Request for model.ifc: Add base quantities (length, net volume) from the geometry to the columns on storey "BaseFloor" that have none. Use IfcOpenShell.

First a look at what the model holds.

```python
import ifcopenshell
import ifcopenshell.util.element
import ifcopenshell.util.unit

model = ifcopenshell.open("model.ifc")
print(model.schema)
for unit_type in ("LENGTHUNIT", "AREAUNIT", "VOLUMEUNIT"):
    print(unit_type, ifcopenshell.util.unit.calculate_unit_scale(model, unit_type))
storey = next(s for s in model.by_type("IfcBuildingStorey") if s.Name == "BaseFloor")
columns = [e for e in ifcopenshell.util.element.get_decomposition(storey) if e.is_a("IfcColumn")]
for e in sorted(columns, key=lambda e: e.id()):
    print(e.id(), e.is_a(), e.Name, list(ifcopenshell.util.element.get_psets(e, qtos_only=True)), sep=" | ")
```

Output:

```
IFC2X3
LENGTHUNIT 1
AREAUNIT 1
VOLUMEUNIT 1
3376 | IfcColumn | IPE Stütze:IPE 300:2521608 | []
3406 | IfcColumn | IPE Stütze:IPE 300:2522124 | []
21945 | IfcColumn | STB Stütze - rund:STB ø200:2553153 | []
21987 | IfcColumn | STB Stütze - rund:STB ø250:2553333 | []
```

```python
import ifcopenshell
import ifcopenshell.api.pset
import ifcopenshell.geom
import ifcopenshell.util.element
import ifcopenshell.util.shape
import ifcopenshell.util.unit

model = ifcopenshell.open("model.ifc")
unit_scale = ifcopenshell.util.unit.calculate_unit_scale(model)
volume_scale = ifcopenshell.util.unit.calculate_unit_scale(model, "VOLUMEUNIT")
settings = ifcopenshell.geom.settings()

storey = next(s for s in model.by_type("IfcBuildingStorey") if s.Name == "BaseFloor")
columns = [e for e in ifcopenshell.util.element.get_decomposition(storey) if e.is_a("IfcColumn")]

for e in sorted(columns, key=lambda e: e.id()):
    if ifcopenshell.util.element.get_psets(e, qtos_only=True, should_inherit=False):
        continue
    # Geometry comes back in metres, in the element's own axes.
    shape = ifcopenshell.geom.create_shape(settings, e)
    values = {
        "Length": ifcopenshell.util.shape.get_z(shape.geometry) / unit_scale,
        "NetVolume": ifcopenshell.util.shape.get_volume(shape.geometry) / volume_scale,
    }
    qto = ifcopenshell.api.pset.add_qto(model, product=e, name="BaseQuantities")
    ifcopenshell.api.pset.edit_qto(model, qto=qto, properties=values)
    print(e.id(), {k: round(v, 3) for k, v in values.items()})

model.write("model-out.ifc")
```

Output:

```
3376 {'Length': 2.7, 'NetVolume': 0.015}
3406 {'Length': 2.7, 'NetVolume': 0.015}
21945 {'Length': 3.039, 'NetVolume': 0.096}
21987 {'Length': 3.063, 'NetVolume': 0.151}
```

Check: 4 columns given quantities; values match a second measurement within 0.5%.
